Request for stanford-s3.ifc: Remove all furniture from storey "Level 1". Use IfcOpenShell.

First a look at what the model holds.

```python
import ifcopenshell
import ifcopenshell.util.element

model = ifcopenshell.open("stanford-s3.ifc")
print(model.schema)
storey = next(s for s in model.by_type("IfcBuildingStorey") if s.Name == "Level 1")
furniture = [e for e in ifcopenshell.util.element.get_decomposition(storey) if e.is_a("IfcFurnishingElement")]
seen = {}
for e in furniture:
    element_type = ifcopenshell.util.element.get_type(e)
    name = element_type.Name if element_type not in (None, e) else None
    seen[name] = seen.get(name, 0) + 1
for name, count in sorted(seen.items(), key=str):
    print(count, "x", name)
```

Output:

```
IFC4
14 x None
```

```python
import ifcopenshell
import ifcopenshell.api.root
import ifcopenshell.util.element

model = ifcopenshell.open("stanford-s3.ifc")

storey = next(s for s in model.by_type("IfcBuildingStorey") if s.Name == "Level 1")
furniture = [e for e in ifcopenshell.util.element.get_decomposition(storey) if e.is_a("IfcFurnishingElement")]

for e in furniture:
    ifcopenshell.api.root.remove_product(model, product=e)
print(len(furniture), "removed")

model.write("stanford-s3_rev.ifc")
```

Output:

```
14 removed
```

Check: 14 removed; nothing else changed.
